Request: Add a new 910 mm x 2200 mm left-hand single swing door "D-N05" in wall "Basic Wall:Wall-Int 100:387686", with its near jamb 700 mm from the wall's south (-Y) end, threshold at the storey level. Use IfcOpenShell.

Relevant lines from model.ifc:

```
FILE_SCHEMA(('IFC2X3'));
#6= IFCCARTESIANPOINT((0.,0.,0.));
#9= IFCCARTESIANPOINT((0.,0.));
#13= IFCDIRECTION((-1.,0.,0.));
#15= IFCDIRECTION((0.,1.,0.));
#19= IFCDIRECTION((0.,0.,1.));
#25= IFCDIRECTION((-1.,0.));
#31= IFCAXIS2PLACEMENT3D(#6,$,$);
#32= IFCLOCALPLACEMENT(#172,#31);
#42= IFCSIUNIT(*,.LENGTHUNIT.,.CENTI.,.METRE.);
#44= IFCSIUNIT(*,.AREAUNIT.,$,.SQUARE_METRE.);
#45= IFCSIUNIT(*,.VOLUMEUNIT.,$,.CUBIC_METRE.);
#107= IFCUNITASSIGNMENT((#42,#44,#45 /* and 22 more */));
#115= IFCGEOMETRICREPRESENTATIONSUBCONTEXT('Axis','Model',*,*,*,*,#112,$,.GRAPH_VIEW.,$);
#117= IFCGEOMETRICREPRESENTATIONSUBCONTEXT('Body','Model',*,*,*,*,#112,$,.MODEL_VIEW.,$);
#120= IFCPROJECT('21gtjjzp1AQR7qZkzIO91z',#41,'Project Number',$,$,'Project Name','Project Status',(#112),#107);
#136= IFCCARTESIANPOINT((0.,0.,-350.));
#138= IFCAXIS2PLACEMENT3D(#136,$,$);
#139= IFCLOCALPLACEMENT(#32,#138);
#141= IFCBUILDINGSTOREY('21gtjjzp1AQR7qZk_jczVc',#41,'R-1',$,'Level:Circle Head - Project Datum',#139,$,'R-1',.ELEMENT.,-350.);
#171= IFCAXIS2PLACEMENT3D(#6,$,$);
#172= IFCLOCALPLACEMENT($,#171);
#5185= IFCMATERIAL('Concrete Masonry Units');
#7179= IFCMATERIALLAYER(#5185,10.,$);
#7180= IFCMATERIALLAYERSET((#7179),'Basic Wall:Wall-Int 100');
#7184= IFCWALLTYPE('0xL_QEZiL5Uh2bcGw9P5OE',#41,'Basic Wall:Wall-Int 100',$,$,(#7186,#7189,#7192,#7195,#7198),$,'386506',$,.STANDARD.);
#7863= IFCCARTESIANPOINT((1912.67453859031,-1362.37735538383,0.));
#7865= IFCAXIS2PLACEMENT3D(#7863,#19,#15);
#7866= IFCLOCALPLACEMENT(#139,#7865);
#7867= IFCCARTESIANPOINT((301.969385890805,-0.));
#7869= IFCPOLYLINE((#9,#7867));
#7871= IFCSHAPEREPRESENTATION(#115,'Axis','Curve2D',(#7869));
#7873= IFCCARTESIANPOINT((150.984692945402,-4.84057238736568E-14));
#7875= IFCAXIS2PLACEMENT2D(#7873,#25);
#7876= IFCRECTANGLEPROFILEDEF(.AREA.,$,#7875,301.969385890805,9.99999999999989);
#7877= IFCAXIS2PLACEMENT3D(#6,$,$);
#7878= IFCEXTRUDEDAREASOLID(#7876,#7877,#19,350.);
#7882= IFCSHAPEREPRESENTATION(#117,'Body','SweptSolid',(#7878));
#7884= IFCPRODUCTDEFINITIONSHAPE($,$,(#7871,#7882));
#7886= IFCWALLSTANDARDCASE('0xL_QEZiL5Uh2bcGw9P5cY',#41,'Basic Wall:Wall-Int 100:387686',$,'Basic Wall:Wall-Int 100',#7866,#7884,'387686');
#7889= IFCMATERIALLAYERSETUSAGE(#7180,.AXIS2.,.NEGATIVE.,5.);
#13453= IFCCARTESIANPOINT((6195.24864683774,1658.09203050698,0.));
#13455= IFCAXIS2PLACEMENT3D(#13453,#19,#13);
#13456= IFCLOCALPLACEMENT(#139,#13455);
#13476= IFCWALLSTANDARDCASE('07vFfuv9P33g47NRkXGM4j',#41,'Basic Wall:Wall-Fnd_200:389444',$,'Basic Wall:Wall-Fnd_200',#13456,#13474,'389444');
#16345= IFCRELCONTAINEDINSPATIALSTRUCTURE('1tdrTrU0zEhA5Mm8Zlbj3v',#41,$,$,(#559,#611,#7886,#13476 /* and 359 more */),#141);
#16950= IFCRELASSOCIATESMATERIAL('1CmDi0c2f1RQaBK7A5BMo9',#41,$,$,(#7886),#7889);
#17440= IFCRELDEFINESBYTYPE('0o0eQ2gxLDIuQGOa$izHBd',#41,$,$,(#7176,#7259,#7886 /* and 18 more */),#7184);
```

```python
import numpy as np
import ifcopenshell
import ifcopenshell.api.feature
import ifcopenshell.api.geometry
import ifcopenshell.api.root
import ifcopenshell.api.spatial
import ifcopenshell.api.type
import ifcopenshell.geom
import ifcopenshell.util.element
import ifcopenshell.util.placement
import ifcopenshell.util.representation
import ifcopenshell.util.shape
import ifcopenshell.util.unit

model = ifcopenshell.open("model.ifc")
unit_scale = ifcopenshell.util.unit.calculate_unit_scale(model)
settings = ifcopenshell.geom.settings()


def volume(element):
    """Net volume in cubic metres, openings subtracted."""
    shape = ifcopenshell.geom.create_shape(settings, element)
    return ifcopenshell.util.shape.get_volume(shape.geometry)


wall = model.by_id(7886)
storey = ifcopenshell.util.element.get_container(wall, ifc_class="IfcBuildingStorey")
context = ifcopenshell.util.representation.get_context(model, "Model", "Body", "MODEL_VIEW")
before = volume(wall)

width, height, from_end, sill = 0.91, 2.2, 0.7, 0.0  # metres

# The wall runs along its own X axis, and the end named is its -X end.
wall_shape = ifcopenshell.geom.create_shape(settings, wall)
x, y, z = ifcopenshell.util.shape.get_vertices(wall_shape.geometry).T
start = x.min() + from_end
face, thickness = float(y.min()), float(y.max() - y.min())
wall_matrix = ifcopenshell.util.placement.get_local_placement(wall.ObjectPlacement)
level = ifcopenshell.util.placement.get_local_placement(storey.ObjectPlacement)[2, 3]


def in_wall(x, y):
    """Placement at x, y metres in the wall's axes, at sill height."""
    matrix = wall_matrix.copy()
    matrix[:, 3] = wall_matrix @ np.array([x / unit_scale, y / unit_scale, 0.0, 1.0])
    matrix[2, 3] = level + sill / unit_scale
    return matrix


# Opening: a box that overshoots both wall faces by 50 mm.
opening = ifcopenshell.api.root.create_entity(model, ifc_class="IfcOpeningElement")
box = ifcopenshell.api.geometry.add_wall_representation(
    model, context=context, length=width, height=height, thickness=thickness + 0.1
)
ifcopenshell.api.geometry.assign_representation(model, product=opening, representation=box)
ifcopenshell.api.geometry.edit_object_placement(model, product=opening, matrix=in_wall(start, face - 0.05), is_si=False)
ifcopenshell.api.feature.add_feature(model, feature=opening, element=wall)

door = ifcopenshell.api.root.create_entity(model, ifc_class="IfcDoor", name="D-N05")
door.OverallWidth, door.OverallHeight = width / unit_scale, height / unit_scale
body = ifcopenshell.api.geometry.add_door_representation(
    model,
    context=context,
    overall_width=door.OverallWidth,
    overall_height=door.OverallHeight,
    operation_type="SINGLE_SWING_LEFT",
    lining_properties={"LiningDepth": thickness / unit_scale, "ThresholdDepth": thickness / unit_scale},
)
ifcopenshell.api.geometry.assign_representation(model, product=door, representation=body)
ifcopenshell.api.spatial.assign_container(model, products=[door], relating_structure=storey)
fills = ifcopenshell.api.feature.add_filling(model, opening=opening, element=door)
fills.OwnerHistory = door.OwnerHistory  # required in IFC2X3

# IFC2X3 keeps the operation on the door style.
style = ifcopenshell.api.root.create_entity(model, ifc_class="IfcDoorStyle", name="D-N05")
style.OperationType, style.ConstructionType = "SINGLE_SWING_LEFT", "NOTDEFINED"
style.ParameterTakesPrecedence = style.Sizeable = False
ifcopenshell.api.type.assign_type(model, related_objects=[door], relating_type=style)

# The lining spans the wall, so the door starts at the wall face.
ifcopenshell.api.geometry.edit_object_placement(model, product=door, matrix=in_wall(start, face), is_si=False)

after = volume(wall)

print(f"wall volume {before:.3f} -> {after:.3f} m3")

model.write("model-out.ifc")
```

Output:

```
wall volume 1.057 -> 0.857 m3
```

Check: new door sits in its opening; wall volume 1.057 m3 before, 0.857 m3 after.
